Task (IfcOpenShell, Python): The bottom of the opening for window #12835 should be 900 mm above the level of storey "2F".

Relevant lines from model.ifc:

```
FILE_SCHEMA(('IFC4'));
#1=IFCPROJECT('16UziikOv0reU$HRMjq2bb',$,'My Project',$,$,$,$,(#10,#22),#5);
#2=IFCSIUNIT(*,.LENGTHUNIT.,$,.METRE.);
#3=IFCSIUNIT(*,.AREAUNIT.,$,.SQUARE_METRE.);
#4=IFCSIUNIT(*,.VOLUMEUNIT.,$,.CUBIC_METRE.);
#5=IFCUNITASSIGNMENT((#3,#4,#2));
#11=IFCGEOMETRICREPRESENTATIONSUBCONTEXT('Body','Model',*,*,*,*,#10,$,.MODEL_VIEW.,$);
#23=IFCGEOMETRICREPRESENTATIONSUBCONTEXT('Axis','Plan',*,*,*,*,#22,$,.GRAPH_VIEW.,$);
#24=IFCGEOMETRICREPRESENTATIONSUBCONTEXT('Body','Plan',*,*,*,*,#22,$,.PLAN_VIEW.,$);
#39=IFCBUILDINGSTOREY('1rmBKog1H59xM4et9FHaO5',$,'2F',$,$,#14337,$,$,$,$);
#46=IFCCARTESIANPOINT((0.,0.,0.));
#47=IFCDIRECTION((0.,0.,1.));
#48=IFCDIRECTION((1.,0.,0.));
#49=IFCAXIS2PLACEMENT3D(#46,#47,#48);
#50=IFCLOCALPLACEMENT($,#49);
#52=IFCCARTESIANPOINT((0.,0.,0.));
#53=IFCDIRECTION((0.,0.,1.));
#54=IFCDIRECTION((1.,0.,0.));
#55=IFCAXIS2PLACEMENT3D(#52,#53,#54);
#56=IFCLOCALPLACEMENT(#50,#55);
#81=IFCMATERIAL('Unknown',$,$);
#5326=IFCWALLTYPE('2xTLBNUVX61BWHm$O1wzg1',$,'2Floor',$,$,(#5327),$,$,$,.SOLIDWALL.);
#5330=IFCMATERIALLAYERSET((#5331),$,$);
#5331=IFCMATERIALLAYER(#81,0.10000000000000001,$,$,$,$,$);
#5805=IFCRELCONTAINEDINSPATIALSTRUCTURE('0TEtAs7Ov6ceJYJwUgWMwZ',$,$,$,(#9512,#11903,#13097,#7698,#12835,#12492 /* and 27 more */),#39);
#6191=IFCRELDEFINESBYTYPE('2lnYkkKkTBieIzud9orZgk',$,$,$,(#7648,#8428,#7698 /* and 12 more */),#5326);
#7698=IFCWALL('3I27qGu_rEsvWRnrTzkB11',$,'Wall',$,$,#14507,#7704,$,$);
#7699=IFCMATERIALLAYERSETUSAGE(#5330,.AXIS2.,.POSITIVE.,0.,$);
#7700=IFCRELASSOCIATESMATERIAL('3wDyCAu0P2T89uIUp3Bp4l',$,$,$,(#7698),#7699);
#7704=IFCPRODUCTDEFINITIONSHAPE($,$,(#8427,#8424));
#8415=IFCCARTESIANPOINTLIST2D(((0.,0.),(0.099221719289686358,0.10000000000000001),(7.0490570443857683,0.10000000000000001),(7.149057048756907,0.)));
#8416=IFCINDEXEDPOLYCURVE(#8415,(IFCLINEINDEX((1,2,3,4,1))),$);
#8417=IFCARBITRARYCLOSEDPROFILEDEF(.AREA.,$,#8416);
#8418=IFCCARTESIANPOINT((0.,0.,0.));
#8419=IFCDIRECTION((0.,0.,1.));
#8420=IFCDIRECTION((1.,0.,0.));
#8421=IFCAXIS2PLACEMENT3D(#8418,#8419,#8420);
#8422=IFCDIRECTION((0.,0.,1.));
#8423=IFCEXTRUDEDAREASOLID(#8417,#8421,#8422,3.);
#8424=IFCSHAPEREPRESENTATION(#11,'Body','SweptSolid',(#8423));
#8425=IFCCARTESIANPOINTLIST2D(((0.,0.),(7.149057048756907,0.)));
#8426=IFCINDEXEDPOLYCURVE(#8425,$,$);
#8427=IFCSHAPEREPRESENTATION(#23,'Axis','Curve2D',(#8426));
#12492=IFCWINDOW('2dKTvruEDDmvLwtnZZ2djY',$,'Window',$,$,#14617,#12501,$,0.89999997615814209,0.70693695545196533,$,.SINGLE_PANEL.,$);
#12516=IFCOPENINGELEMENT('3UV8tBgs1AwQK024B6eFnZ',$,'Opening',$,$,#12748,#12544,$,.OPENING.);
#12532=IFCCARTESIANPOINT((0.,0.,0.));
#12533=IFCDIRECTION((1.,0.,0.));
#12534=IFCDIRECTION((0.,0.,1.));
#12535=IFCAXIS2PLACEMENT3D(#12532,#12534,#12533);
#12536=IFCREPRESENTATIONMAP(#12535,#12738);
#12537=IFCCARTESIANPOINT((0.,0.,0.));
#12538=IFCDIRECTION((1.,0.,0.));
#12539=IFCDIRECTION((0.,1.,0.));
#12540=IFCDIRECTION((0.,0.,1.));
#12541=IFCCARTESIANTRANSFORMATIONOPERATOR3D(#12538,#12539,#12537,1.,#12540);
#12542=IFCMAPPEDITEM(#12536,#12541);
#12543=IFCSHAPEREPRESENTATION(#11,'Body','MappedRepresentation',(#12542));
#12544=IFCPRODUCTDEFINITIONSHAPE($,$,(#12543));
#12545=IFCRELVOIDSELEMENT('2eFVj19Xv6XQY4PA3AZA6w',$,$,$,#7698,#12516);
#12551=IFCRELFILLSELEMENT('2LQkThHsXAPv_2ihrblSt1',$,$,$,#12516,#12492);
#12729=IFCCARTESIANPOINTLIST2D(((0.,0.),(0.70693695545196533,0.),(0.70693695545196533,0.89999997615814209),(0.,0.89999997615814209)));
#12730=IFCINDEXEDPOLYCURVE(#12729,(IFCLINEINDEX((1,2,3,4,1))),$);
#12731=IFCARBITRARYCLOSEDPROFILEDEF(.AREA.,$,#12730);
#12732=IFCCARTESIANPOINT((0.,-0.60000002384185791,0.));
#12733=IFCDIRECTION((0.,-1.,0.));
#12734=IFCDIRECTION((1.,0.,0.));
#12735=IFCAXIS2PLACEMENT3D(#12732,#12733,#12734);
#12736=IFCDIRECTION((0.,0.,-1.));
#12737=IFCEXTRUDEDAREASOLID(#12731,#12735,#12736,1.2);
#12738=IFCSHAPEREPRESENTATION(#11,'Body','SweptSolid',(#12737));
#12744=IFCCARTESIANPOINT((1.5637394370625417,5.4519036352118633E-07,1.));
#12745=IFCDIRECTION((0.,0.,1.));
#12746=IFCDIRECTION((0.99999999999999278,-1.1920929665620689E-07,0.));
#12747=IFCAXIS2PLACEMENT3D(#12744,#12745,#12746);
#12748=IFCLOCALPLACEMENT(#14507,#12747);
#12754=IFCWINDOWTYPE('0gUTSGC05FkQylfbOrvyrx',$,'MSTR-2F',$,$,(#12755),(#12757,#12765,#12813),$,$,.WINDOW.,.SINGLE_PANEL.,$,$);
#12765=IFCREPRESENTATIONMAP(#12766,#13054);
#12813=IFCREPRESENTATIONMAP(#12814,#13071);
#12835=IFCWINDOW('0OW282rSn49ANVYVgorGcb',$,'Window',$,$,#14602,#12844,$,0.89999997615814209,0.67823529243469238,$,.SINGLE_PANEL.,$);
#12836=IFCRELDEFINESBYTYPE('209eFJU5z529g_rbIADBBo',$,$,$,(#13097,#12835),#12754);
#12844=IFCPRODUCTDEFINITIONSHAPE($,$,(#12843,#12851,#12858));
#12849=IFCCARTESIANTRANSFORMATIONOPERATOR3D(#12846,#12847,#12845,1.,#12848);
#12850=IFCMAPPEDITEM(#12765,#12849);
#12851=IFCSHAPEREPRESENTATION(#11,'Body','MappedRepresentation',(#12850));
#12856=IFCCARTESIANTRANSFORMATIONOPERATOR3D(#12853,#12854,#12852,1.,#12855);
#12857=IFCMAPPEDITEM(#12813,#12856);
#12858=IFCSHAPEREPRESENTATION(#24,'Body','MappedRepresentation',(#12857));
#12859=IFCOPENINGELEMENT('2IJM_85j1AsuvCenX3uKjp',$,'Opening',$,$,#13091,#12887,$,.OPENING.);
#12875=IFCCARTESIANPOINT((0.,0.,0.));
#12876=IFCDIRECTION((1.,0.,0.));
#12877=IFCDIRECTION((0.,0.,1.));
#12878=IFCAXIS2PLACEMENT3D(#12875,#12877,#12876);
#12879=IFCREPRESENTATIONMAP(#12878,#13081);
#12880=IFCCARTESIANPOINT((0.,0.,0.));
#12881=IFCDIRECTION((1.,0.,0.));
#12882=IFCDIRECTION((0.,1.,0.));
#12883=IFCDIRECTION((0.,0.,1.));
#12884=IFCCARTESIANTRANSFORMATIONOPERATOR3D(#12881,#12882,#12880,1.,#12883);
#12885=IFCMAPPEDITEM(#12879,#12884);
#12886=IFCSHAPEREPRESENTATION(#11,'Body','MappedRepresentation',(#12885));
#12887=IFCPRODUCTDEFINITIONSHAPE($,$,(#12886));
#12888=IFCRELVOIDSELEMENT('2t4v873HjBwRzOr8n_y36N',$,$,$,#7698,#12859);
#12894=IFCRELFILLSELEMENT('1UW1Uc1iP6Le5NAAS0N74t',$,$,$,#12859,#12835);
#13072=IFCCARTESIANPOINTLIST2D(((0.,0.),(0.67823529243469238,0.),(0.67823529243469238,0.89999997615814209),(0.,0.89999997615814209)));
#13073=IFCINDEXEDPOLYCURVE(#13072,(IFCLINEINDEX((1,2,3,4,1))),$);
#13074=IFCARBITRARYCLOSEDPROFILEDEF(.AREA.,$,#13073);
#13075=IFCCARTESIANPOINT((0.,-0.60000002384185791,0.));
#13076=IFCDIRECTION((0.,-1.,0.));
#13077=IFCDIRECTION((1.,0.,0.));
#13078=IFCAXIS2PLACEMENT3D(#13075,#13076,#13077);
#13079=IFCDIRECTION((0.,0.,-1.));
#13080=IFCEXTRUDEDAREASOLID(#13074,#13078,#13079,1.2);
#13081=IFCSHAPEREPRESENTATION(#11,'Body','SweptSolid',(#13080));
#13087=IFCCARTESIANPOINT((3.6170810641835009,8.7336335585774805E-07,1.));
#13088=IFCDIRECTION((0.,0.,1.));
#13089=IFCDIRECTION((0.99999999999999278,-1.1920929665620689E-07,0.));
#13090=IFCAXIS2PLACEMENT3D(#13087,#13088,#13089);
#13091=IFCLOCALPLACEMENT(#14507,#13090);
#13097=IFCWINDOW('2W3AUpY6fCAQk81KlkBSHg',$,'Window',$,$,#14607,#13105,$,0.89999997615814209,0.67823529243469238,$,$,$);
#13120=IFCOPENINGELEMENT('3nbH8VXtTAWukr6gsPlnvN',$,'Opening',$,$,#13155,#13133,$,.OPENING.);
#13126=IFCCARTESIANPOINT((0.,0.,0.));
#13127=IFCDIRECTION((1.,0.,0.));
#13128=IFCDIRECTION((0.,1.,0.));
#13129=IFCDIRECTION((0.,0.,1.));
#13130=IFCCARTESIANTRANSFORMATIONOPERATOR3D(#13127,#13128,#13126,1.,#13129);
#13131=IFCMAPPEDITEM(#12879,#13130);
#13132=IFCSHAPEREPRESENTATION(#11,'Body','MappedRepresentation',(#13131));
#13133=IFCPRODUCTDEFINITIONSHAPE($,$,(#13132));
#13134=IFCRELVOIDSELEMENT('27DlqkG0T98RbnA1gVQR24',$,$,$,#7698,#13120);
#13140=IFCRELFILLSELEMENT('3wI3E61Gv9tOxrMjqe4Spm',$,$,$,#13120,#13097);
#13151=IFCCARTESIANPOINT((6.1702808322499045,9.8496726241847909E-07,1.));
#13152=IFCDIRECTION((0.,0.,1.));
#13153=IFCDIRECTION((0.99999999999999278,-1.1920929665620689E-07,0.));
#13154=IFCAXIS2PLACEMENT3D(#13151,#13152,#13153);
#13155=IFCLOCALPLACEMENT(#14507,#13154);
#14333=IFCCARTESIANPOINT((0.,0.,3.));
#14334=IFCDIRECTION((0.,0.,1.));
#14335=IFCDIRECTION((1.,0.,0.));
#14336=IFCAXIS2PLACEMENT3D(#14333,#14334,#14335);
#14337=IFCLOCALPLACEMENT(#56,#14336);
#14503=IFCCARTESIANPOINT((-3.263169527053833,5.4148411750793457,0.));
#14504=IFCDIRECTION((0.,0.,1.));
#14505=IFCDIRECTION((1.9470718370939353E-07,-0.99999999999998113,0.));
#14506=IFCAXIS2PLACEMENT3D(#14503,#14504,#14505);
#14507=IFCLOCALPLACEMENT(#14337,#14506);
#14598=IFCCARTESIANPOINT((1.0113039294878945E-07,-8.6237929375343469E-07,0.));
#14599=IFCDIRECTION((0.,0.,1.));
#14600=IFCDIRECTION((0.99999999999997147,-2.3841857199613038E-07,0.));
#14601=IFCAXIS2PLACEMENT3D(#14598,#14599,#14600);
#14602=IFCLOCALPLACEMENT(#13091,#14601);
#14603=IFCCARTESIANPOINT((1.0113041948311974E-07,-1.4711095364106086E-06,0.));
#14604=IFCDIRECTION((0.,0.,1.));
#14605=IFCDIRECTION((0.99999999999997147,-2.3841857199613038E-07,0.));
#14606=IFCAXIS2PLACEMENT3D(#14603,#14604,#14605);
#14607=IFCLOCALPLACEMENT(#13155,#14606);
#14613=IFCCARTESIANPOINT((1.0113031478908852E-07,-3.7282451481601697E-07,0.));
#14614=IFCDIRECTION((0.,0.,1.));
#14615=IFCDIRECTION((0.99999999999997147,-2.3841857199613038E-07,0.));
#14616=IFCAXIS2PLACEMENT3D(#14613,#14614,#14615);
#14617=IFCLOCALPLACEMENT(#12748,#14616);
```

```python
import numpy as np
import ifcopenshell
import ifcopenshell.api.geometry
import ifcopenshell.geom
import ifcopenshell.util.element
import ifcopenshell.util.placement
import ifcopenshell.util.shape
import ifcopenshell.util.unit

model = ifcopenshell.open("model.ifc")
unit_scale = ifcopenshell.util.unit.calculate_unit_scale(model)

window = model.by_id(12835)
opening = window.FillsVoids[0].RelatingOpeningElement
storey = ifcopenshell.util.element.get_container(window, ifc_class="IfcBuildingStorey")
level = ifcopenshell.util.placement.get_local_placement(storey.ObjectPlacement)[2, 3]

# The opening's origin need not be at the sill, so measure its lowest point.
shape = ifcopenshell.geom.create_shape(ifcopenshell.geom.settings(), opening)
bottom = ifcopenshell.util.shape.get_shape_bottom_elevation(shape, shape.geometry) / unit_scale
dz = level + 0.9 / unit_scale - bottom

shift = np.array([0.0, 0.0, dz])
# The window is placed relative to its opening, so it follows when the opening moves.
matrix = ifcopenshell.util.placement.get_local_placement(opening.ObjectPlacement)
matrix[:3, 3] += shift
ifcopenshell.api.geometry.edit_object_placement(
    model, product=opening, matrix=matrix, is_si=False, should_transform_children=True
)

print(f"moved by {dz * unit_scale:+.3f} m")

model.write("model-out.ifc")
```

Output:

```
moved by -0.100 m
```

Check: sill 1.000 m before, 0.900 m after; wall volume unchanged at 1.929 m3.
